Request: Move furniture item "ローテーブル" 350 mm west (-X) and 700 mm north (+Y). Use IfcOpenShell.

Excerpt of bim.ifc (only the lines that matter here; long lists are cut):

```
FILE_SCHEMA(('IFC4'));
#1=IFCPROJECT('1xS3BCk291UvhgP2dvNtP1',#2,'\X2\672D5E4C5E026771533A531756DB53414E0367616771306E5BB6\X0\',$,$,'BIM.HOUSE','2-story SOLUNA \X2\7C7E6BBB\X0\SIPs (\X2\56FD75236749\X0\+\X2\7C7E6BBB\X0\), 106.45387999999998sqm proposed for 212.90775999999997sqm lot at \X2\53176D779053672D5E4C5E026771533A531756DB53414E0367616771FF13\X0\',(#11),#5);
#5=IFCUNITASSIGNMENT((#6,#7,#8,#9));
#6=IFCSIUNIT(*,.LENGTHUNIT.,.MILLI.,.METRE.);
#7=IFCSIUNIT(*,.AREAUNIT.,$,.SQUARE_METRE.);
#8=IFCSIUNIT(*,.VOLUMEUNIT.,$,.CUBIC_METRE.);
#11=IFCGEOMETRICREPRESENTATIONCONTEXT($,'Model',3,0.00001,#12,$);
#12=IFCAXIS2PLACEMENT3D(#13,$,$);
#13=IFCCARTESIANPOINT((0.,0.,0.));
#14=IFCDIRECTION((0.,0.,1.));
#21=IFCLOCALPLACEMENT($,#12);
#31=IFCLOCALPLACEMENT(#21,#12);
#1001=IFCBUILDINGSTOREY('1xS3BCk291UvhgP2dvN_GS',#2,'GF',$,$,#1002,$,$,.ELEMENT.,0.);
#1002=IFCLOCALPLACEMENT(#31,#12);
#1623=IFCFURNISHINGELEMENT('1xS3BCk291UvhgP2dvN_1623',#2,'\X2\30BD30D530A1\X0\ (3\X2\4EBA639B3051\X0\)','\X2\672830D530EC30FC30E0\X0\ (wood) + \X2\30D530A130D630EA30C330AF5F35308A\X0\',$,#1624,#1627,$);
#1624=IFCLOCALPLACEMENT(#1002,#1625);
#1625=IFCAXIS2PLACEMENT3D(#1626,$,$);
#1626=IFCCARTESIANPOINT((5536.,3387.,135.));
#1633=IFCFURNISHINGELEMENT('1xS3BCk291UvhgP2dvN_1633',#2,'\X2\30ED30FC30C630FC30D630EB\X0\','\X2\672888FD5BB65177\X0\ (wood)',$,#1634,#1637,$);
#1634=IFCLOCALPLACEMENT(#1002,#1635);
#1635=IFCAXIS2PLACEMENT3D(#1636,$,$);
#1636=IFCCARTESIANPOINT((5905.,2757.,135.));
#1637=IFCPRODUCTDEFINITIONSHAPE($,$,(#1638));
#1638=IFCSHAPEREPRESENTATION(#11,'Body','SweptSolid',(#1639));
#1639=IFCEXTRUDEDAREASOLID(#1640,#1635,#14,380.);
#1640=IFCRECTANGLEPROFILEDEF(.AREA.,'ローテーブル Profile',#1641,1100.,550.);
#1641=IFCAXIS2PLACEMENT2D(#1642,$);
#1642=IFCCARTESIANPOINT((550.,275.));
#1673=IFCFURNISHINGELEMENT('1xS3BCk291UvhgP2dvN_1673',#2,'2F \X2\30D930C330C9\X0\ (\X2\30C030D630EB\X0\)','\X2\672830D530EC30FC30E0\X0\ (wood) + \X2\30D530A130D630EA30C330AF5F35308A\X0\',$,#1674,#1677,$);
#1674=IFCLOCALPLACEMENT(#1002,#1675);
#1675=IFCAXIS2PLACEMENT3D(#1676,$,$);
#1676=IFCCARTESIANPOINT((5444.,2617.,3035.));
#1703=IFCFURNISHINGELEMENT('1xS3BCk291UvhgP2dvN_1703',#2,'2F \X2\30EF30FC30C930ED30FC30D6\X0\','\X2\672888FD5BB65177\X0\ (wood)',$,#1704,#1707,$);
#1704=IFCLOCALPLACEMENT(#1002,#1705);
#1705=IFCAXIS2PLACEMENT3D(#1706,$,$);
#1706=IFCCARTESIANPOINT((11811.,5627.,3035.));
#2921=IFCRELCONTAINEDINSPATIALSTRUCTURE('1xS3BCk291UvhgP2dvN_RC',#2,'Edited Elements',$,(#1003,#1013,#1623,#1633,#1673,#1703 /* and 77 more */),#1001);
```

```python
import ifcopenshell
import ifcopenshell.api.geometry
import ifcopenshell.util.placement

model = ifcopenshell.open("bim.ifc")

item = model.by_id(1633)
matrix = ifcopenshell.util.placement.get_local_placement(item.ObjectPlacement)
matrix[0, 3] -= 350.0
matrix[1, 3] += 700.0
ifcopenshell.api.geometry.edit_object_placement(model, product=item, matrix=matrix, is_si=False)

print(ifcopenshell.util.placement.get_local_placement(item.ObjectPlacement).round(3) + 0.0)

model.write("bim_updated.ifc")
```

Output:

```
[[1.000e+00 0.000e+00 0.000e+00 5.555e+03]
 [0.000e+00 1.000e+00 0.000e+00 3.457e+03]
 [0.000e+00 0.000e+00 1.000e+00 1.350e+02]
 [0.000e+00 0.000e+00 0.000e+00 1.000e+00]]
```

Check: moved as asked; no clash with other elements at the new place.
